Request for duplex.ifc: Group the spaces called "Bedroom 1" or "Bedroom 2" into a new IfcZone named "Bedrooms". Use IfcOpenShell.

First a look at what the model holds.

```python
import ifcopenshell

model = ifcopenshell.open("duplex.ifc")
print(model.schema)
seen = {}
for space in model.by_type("IfcSpace"):
    seen[space.LongName] = seen.get(space.LongName, 0) + 1
for name, count in sorted(seen.items(), key=str):
    print(count, "x", name)
print("zones:", [z.Name for z in model.by_type("IfcZone")][:20])
```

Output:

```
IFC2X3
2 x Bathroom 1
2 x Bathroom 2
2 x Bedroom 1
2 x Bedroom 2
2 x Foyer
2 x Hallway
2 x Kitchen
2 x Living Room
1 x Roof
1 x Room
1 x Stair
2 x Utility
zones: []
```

```python
import ifcopenshell
import ifcopenshell.api.group
import ifcopenshell.api.root

model = ifcopenshell.open("duplex.ifc")

names = {"Bedroom 1", "Bedroom 2"}
spaces = [s for s in model.by_type("IfcSpace") if s.LongName in names]

zone = ifcopenshell.api.root.create_entity(model, ifc_class="IfcZone", name="Bedrooms")
ifcopenshell.api.group.assign_group(model, products=spaces, group=zone)
print(len(spaces), "spaces in", zone.Name)

model.write("duplex_edited.ifc")
```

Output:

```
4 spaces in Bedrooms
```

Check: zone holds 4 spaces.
